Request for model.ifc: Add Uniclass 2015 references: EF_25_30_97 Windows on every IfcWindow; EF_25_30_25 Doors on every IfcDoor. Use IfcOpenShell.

First a look at what the model holds.

```python
import ifcopenshell

model = ifcopenshell.open("model.ifc")
print(model.schema)
print("classifications:", [c.Name for c in model.by_type("IfcClassification")])
for ifc_class in ("IfcDoor", "IfcRoof", "IfcStair", "IfcWall", "IfcWindow"):
    print(ifc_class, len(model.by_type(ifc_class)))
```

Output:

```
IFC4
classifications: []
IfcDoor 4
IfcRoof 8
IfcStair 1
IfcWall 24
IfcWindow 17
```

```python
import ifcopenshell
import ifcopenshell.api.classification

model = ifcopenshell.open("model.ifc")

system = ifcopenshell.api.classification.add_classification(model, classification="Uniclass 2015")

codes = {
    "IfcWindow": ("EF_25_30_97", "Windows"),
    "IfcDoor": ("EF_25_30_25", "Doors"),
}
for ifc_class, (code, name) in codes.items():
    products = model.by_type(ifc_class)
    ifcopenshell.api.classification.add_reference(
        model, products=products, classification=system, identification=code, name=name
    )
    print(code, len(products))

model.write("model_edited.ifc")
```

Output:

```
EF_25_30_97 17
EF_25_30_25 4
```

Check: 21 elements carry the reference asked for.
